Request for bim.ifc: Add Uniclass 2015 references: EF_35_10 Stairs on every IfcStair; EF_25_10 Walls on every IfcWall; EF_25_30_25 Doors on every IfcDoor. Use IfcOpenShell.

First a look at what the model holds.

```python
import ifcopenshell

model = ifcopenshell.open("bim.ifc")
print(model.schema)
print("classifications:", [c.Name for c in model.by_type("IfcClassification")])
for ifc_class in ("IfcDoor", "IfcRoof", "IfcStair", "IfcWall", "IfcWindow"):
    print(ifc_class, len(model.by_type(ifc_class)))
```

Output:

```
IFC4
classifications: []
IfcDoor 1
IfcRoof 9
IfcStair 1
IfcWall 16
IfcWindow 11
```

```python
import ifcopenshell
import ifcopenshell.api.classification

model = ifcopenshell.open("bim.ifc")

system = ifcopenshell.api.classification.add_classification(model, classification="Uniclass 2015")

codes = {
    "IfcStair": ("EF_35_10", "Stairs"),
    "IfcWall": ("EF_25_10", "Walls"),
    "IfcDoor": ("EF_25_30_25", "Doors"),
}
for ifc_class, (code, name) in codes.items():
    products = model.by_type(ifc_class)
    ifcopenshell.api.classification.add_reference(
        model, products=products, classification=system, identification=code, name=name
    )
    print(code, len(products))

model.write("bim_edited.ifc")
```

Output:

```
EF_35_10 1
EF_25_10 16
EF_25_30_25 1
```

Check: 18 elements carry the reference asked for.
